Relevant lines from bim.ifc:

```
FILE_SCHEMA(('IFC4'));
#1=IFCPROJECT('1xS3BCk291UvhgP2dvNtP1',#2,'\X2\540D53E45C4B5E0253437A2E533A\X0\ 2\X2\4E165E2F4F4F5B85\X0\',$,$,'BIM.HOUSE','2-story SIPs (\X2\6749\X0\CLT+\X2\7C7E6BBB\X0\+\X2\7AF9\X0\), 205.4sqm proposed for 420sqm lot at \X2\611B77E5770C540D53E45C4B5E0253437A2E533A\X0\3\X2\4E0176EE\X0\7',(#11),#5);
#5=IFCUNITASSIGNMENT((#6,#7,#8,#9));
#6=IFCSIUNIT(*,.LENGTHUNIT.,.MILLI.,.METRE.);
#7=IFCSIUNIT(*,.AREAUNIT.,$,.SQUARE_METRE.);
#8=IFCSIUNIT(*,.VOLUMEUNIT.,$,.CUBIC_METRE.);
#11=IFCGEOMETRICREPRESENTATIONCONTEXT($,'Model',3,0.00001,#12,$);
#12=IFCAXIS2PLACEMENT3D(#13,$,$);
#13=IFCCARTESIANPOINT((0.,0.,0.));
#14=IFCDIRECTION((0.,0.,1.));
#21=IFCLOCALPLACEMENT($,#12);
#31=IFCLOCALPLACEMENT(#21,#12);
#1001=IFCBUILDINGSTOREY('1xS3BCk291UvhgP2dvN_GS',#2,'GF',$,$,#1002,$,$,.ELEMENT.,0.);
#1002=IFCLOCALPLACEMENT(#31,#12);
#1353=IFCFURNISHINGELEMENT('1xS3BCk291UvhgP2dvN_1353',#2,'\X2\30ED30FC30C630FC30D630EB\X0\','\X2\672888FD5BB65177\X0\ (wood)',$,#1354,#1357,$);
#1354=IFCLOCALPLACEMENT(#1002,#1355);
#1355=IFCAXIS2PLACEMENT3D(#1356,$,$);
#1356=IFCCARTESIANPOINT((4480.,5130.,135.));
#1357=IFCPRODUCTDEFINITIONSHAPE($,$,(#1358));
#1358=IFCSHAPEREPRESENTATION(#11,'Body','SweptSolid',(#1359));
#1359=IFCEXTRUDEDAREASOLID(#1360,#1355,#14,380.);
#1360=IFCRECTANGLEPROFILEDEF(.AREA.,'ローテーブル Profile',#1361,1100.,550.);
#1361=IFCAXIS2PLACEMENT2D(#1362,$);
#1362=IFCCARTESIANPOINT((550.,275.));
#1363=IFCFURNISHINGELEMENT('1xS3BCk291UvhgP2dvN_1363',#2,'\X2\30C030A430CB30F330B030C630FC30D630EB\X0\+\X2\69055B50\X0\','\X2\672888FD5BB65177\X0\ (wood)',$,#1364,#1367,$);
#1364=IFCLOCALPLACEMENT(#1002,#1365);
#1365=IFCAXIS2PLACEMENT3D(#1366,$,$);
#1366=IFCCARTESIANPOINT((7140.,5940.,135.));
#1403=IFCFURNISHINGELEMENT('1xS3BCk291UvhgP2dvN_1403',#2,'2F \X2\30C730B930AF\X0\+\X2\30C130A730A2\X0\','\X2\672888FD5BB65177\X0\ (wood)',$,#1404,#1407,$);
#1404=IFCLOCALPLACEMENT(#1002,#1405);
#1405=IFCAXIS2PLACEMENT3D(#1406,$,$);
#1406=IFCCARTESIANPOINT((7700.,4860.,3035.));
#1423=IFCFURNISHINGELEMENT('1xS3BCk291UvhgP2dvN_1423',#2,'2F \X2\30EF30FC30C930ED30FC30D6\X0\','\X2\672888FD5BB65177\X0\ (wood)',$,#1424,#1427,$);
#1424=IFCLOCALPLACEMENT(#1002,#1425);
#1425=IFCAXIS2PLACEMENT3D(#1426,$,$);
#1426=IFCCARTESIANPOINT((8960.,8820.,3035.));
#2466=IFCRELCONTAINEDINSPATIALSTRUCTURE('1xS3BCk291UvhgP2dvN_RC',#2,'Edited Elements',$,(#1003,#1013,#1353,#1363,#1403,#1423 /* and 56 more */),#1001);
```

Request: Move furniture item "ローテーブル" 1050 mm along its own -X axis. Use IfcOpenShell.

```python
import ifcopenshell
import ifcopenshell.api.geometry
import ifcopenshell.util.placement
import ifcopenshell.util.unit

model = ifcopenshell.open("bim.ifc")
unit_scale = ifcopenshell.util.unit.calculate_unit_scale(model)

item = model.by_id(1353)
matrix = ifcopenshell.util.placement.get_local_placement(item.ObjectPlacement)
matrix[:3, 3] -= matrix[:3, 0] * 1.05 / unit_scale
ifcopenshell.api.geometry.edit_object_placement(model, product=item, matrix=matrix, is_si=False)

print(ifcopenshell.util.placement.get_local_placement(item.ObjectPlacement).round(3) + 0.0)

model.write("bim_rev.ifc")
```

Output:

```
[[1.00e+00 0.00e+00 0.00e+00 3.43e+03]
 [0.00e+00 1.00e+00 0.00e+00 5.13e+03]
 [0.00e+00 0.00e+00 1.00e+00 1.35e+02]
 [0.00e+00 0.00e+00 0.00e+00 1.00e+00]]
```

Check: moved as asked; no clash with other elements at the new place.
